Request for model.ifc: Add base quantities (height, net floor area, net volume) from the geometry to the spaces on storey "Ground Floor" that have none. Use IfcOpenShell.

First a look at what the model holds.

```python
import ifcopenshell
import ifcopenshell.util.element
import ifcopenshell.util.unit

model = ifcopenshell.open("model.ifc")
print(model.schema)
for unit_type in ("LENGTHUNIT", "AREAUNIT", "VOLUMEUNIT"):
    print(unit_type, ifcopenshell.util.unit.calculate_unit_scale(model, unit_type))
storey = next(s for s in model.by_type("IfcBuildingStorey") if s.Name == "Ground Floor")
spaces = [e for e in ifcopenshell.util.element.get_decomposition(storey) if e.is_a("IfcSpace")]
for e in sorted(spaces, key=lambda e: e.id()):
    print(e.id(), e.is_a(), e.Name, list(ifcopenshell.util.element.get_psets(e, qtos_only=True)), sep=" | ")
```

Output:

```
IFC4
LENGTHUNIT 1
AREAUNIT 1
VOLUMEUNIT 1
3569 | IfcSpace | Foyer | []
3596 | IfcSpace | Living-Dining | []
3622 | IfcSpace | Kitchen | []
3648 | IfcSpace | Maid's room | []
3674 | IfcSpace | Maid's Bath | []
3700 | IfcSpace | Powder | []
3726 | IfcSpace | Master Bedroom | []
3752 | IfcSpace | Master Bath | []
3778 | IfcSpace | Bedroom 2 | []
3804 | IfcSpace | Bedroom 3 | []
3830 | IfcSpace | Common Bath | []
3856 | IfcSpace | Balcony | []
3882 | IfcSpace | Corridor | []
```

```python
import ifcopenshell
import ifcopenshell.api.pset
import ifcopenshell.geom
import ifcopenshell.util.element
import ifcopenshell.util.shape
import ifcopenshell.util.unit

model = ifcopenshell.open("model.ifc")
unit_scale = ifcopenshell.util.unit.calculate_unit_scale(model)
area_scale = ifcopenshell.util.unit.calculate_unit_scale(model, "AREAUNIT")
volume_scale = ifcopenshell.util.unit.calculate_unit_scale(model, "VOLUMEUNIT")
settings = ifcopenshell.geom.settings()

storey = next(s for s in model.by_type("IfcBuildingStorey") if s.Name == "Ground Floor")
spaces = [e for e in ifcopenshell.util.element.get_decomposition(storey) if e.is_a("IfcSpace")]

for e in sorted(spaces, key=lambda e: e.id()):
    if ifcopenshell.util.element.get_psets(e, qtos_only=True, should_inherit=False):
        continue
    # Geometry comes back in metres, in the element's own axes.
    shape = ifcopenshell.geom.create_shape(settings, e)
    values = {
        "Height": ifcopenshell.util.shape.get_z(shape.geometry) / unit_scale,
        "NetFloorArea": ifcopenshell.util.shape.get_footprint_area(shape.geometry) / area_scale,
        "NetVolume": ifcopenshell.util.shape.get_volume(shape.geometry) / volume_scale,
    }
    qto = ifcopenshell.api.pset.add_qto(model, product=e, name="Qto_SpaceBaseQuantities")
    ifcopenshell.api.pset.edit_qto(model, qto=qto, properties=values)
    print(e.id(), {k: round(v, 3) for k, v in values.items()})

model.write("model_edited.ifc")
```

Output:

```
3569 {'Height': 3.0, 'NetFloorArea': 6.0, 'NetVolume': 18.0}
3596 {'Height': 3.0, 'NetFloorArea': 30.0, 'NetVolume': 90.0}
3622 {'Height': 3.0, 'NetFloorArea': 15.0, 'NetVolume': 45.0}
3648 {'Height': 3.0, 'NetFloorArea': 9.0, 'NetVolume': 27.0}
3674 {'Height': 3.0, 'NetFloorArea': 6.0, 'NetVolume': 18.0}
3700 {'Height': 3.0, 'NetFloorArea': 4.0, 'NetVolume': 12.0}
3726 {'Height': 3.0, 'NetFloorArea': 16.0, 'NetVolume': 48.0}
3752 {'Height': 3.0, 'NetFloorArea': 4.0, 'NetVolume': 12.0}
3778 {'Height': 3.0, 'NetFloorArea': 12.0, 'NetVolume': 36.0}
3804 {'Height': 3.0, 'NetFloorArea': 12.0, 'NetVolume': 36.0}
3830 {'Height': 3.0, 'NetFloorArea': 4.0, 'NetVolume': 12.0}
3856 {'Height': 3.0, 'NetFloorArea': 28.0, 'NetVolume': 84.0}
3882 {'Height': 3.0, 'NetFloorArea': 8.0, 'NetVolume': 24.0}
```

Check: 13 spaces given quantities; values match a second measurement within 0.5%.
